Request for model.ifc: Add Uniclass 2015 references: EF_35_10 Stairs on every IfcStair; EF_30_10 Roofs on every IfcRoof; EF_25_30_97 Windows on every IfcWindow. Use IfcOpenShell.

First a look at what the model holds.

```python
import ifcopenshell

model = ifcopenshell.open("model.ifc")
print(model.schema)
print("classifications:", [c.Name for c in model.by_type("IfcClassification")])
for ifc_class in ("IfcDoor", "IfcRoof", "IfcStair", "IfcWall", "IfcWindow"):
    print(ifc_class, len(model.by_type(ifc_class)))
```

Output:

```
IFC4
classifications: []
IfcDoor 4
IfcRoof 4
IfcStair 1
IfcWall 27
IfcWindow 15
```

```python
import ifcopenshell
import ifcopenshell.api.classification

model = ifcopenshell.open("model.ifc")

system = ifcopenshell.api.classification.add_classification(model, classification="Uniclass 2015")

codes = {
    "IfcStair": ("EF_35_10", "Stairs"),
    "IfcRoof": ("EF_30_10", "Roofs"),
    "IfcWindow": ("EF_25_30_97", "Windows"),
}
for ifc_class, (code, name) in codes.items():
    products = model.by_type(ifc_class)
    ifcopenshell.api.classification.add_reference(
        model, products=products, classification=system, identification=code, name=name
    )
    print(code, len(products))

model.write("model_rev.ifc")
```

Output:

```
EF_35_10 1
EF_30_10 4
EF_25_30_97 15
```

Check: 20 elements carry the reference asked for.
